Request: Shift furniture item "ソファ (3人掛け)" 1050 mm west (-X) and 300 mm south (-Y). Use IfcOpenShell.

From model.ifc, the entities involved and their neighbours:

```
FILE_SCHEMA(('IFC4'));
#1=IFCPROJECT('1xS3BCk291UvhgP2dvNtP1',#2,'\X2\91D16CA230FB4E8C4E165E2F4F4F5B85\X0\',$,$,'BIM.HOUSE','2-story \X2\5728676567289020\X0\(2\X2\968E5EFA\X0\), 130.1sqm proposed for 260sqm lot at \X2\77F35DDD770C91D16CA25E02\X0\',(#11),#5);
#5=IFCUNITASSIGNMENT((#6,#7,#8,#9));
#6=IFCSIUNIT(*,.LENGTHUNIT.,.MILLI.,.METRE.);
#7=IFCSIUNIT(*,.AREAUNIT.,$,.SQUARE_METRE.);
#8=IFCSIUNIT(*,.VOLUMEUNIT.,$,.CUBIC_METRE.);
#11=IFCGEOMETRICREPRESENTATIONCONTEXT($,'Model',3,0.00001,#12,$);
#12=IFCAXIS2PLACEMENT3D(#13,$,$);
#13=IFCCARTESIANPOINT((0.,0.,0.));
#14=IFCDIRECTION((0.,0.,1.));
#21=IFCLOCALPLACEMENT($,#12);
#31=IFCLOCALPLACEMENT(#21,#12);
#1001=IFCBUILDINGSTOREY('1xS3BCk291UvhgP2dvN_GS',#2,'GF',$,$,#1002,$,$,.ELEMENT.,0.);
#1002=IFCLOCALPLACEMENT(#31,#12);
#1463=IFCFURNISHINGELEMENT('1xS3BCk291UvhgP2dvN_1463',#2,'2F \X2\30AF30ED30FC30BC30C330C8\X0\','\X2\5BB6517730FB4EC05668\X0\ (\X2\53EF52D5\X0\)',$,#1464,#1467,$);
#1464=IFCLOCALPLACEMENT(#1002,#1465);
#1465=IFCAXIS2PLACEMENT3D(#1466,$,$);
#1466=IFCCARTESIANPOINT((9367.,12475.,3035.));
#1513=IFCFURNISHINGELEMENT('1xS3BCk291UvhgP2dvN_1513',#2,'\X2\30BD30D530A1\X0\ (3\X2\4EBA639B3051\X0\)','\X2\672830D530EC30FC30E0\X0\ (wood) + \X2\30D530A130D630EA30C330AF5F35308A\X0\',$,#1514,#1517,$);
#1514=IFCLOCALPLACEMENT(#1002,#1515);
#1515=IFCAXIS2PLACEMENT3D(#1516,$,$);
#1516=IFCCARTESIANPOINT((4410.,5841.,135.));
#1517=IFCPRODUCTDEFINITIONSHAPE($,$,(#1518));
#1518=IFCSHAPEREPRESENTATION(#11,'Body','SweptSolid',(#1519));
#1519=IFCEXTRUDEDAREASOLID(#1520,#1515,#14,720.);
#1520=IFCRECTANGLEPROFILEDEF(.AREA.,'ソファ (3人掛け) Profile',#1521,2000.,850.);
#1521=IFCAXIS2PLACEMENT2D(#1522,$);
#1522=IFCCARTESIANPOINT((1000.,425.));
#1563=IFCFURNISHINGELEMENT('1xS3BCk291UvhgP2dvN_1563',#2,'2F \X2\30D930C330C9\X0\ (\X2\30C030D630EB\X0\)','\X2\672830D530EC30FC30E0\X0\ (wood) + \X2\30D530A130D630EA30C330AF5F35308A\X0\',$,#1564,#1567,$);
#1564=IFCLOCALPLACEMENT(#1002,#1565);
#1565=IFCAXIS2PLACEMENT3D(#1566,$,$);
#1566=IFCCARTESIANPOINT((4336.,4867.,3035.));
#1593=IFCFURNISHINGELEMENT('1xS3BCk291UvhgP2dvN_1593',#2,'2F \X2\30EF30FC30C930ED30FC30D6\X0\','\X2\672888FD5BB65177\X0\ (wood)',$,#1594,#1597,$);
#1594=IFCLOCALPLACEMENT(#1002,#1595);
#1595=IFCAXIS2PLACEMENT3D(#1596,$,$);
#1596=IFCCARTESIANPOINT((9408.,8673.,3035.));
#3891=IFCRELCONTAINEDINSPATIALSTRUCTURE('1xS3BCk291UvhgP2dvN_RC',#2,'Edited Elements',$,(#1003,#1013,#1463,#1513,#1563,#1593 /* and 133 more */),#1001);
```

```python
import ifcopenshell
import ifcopenshell.api.geometry
import ifcopenshell.util.placement
import ifcopenshell.util.unit

model = ifcopenshell.open("model.ifc")
unit_scale = ifcopenshell.util.unit.calculate_unit_scale(model)

item = model.by_guid("1xS3BCk291UvhgP2dvN_1513")
matrix = ifcopenshell.util.placement.get_local_placement(item.ObjectPlacement)
matrix[0, 3] -= 1.05 / unit_scale
matrix[1, 3] -= 0.3 / unit_scale
ifcopenshell.api.geometry.edit_object_placement(model, product=item, matrix=matrix, is_si=False)

print(ifcopenshell.util.placement.get_local_placement(item.ObjectPlacement).round(3) + 0.0)

model.write("model_v2.ifc")
```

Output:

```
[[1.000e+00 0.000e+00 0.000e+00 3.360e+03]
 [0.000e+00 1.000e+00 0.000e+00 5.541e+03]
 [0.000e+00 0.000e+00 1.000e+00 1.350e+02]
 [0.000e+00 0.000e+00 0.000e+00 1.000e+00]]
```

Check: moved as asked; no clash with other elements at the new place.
